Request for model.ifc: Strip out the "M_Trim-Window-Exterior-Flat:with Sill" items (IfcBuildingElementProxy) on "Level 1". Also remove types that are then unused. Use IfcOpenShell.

First a look at what the model holds.

```python
import ifcopenshell
import ifcopenshell.util.element

model = ifcopenshell.open("model.ifc")
print(model.schema)
storey = next(s for s in model.by_type("IfcBuildingStorey") if s.Name == "Level 1")
proxies = [e for e in ifcopenshell.util.element.get_decomposition(storey) if e.is_a("IfcBuildingElementProxy")]
seen = {}
for e in proxies:
    element_type = ifcopenshell.util.element.get_type(e)
    name = element_type.Name if element_type not in (None, e) else None
    seen[name] = seen.get(name, 0) + 1
for name, count in sorted(seen.items(), key=str):
    print(count, "x", name)
```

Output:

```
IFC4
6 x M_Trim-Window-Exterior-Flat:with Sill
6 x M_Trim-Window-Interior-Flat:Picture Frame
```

```python
import ifcopenshell
import ifcopenshell.api.root
import ifcopenshell.util.element

model = ifcopenshell.open("model.ifc")

storey = next(s for s in model.by_type("IfcBuildingStorey") if s.Name == "Level 1")
proxies = [e for e in ifcopenshell.util.element.get_decomposition(storey) if e.is_a("IfcBuildingElementProxy")]
targets = [e for e in proxies if (t := ifcopenshell.util.element.get_type(e)) not in (None, e) and t.Name == "M_Trim-Window-Exterior-Flat:with Sill"]
types = {ifcopenshell.util.element.get_type(e) for e in targets} - {None, *targets}

for e in targets:
    ifcopenshell.api.root.remove_product(model, product=e)
print(len(targets), "removed")

unused = [t for t in types if not ifcopenshell.util.element.get_types(t)]
for t in unused:
    ifcopenshell.api.root.remove_product(model, product=t)
print(len(unused), "unused types removed")

model.write("model_updated.ifc")
```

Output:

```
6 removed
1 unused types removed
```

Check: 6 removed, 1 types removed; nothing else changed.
